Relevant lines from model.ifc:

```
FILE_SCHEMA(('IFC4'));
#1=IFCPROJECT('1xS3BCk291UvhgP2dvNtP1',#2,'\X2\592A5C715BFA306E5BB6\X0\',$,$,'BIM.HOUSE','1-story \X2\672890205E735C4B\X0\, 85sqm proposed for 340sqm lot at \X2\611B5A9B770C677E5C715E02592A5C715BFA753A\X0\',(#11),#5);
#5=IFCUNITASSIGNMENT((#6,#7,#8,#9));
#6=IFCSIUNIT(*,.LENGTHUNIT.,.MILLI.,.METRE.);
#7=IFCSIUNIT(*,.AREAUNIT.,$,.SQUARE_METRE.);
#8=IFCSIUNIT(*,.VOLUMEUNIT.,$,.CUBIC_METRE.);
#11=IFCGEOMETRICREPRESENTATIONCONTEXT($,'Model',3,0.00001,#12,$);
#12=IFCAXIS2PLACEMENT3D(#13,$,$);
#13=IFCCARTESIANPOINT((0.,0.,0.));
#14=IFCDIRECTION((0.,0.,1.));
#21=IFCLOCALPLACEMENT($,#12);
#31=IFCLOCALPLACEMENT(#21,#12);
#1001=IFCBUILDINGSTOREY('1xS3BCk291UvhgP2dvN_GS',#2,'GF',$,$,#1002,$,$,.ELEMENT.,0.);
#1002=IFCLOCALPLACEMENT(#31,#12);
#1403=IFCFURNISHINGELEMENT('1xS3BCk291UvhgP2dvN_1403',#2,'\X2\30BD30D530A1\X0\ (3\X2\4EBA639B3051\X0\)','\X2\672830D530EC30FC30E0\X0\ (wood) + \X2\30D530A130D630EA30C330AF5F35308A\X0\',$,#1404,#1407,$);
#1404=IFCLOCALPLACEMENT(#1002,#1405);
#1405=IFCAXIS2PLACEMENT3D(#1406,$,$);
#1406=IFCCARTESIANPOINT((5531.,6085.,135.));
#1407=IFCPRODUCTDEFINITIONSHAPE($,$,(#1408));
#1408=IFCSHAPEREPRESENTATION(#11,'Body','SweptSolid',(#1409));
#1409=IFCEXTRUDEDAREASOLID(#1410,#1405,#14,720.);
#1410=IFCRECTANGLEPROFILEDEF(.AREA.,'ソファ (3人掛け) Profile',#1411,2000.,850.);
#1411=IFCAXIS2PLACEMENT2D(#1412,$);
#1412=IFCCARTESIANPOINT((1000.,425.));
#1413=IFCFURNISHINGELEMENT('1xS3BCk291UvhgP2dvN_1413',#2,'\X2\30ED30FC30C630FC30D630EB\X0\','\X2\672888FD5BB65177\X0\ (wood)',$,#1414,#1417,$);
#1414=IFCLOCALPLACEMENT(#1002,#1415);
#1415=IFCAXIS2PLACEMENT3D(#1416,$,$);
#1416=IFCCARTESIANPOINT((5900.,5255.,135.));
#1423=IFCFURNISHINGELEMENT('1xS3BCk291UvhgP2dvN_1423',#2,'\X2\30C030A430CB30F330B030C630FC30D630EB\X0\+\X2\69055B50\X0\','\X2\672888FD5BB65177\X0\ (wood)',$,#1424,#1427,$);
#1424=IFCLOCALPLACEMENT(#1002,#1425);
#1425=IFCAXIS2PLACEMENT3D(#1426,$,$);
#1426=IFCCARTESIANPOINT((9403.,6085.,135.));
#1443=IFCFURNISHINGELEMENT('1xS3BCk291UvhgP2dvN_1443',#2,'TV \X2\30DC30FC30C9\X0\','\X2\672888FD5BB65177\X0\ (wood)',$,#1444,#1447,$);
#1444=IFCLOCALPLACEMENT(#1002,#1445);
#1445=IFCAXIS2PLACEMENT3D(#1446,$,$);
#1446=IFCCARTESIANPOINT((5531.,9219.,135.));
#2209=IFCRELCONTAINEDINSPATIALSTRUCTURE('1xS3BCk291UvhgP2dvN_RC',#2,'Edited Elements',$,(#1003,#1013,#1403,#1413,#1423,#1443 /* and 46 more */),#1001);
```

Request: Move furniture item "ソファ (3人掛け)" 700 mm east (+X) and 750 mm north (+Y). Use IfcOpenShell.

```python
import ifcopenshell
import ifcopenshell.api.geometry
import ifcopenshell.util.placement

model = ifcopenshell.open("model.ifc")

item = model.by_guid("1xS3BCk291UvhgP2dvN_1403")
matrix = ifcopenshell.util.placement.get_local_placement(item.ObjectPlacement)
matrix[0, 3] += 700.0
matrix[1, 3] += 750.0
ifcopenshell.api.geometry.edit_object_placement(model, product=item, matrix=matrix, is_si=False)

print(ifcopenshell.util.placement.get_local_placement(item.ObjectPlacement).round(3) + 0.0)

model.write("model_rev.ifc")
```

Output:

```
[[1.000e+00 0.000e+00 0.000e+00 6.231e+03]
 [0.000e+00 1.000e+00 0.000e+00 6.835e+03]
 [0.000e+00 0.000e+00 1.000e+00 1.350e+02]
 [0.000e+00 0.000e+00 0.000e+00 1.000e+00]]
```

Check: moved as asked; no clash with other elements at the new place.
